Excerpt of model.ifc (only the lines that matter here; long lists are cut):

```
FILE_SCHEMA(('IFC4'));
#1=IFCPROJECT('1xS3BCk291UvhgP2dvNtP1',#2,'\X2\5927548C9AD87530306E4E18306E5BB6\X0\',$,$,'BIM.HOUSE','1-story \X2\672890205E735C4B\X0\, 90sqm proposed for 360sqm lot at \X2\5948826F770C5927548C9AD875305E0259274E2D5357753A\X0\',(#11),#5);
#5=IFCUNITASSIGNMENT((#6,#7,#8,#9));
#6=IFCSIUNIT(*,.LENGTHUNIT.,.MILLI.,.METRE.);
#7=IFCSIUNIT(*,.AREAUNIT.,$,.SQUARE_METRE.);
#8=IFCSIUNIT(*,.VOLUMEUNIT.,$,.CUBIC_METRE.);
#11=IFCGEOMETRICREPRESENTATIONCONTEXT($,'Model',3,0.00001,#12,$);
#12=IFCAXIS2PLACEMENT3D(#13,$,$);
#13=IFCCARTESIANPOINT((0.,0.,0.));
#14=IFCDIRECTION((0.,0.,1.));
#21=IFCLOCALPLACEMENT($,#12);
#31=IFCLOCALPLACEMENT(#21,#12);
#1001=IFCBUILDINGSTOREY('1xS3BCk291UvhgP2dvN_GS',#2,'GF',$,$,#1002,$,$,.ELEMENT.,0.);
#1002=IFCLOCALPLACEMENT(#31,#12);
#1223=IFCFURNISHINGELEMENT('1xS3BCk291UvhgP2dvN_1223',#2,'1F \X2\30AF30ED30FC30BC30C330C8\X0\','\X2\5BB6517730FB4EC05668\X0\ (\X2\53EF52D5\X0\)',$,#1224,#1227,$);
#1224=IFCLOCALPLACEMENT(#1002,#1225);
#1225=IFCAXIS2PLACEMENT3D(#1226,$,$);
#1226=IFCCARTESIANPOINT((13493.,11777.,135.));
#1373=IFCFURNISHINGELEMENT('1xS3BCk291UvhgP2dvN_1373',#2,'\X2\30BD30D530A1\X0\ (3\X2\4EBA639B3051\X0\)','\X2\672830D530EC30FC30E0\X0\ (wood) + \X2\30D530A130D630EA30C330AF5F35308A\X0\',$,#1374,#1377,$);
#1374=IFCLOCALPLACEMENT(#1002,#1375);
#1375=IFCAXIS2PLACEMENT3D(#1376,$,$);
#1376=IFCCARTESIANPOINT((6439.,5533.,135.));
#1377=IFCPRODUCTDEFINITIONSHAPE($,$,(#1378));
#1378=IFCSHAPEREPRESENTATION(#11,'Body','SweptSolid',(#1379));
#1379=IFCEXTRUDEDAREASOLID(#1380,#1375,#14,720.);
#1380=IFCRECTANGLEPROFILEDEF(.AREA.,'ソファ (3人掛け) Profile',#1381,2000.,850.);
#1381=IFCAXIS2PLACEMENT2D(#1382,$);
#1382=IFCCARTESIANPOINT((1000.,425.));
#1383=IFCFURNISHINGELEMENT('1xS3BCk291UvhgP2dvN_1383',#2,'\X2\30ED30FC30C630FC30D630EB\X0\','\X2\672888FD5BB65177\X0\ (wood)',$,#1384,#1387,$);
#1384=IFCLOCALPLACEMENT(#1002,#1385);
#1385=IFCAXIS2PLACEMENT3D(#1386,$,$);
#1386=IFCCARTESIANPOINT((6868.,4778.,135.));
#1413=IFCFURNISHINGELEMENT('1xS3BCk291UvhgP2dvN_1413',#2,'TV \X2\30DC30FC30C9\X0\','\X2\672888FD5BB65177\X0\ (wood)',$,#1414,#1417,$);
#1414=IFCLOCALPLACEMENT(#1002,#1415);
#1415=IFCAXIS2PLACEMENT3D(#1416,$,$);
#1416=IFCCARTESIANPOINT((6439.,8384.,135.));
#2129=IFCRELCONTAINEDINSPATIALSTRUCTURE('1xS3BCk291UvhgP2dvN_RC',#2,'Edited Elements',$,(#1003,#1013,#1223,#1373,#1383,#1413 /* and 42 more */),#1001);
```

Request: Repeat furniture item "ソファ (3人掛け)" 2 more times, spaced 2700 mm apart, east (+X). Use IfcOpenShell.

```python
import numpy as np
import ifcopenshell
import ifcopenshell.api.geometry
import ifcopenshell.api.root
import ifcopenshell.util.element
import ifcopenshell.util.placement
import ifcopenshell.util.unit

model = ifcopenshell.open("model.ifc")
unit_scale = ifcopenshell.util.unit.calculate_unit_scale(model)


def reuse_history(source, copy):
    """copy_class also copies each property set's owner history, people and application; keep the originals."""
    for rel in copy.IsDefinedBy:
        if rel.is_a("IfcRelDefinesByProperties") and (history := rel.RelatingPropertyDefinition.OwnerHistory):
            rel.RelatingPropertyDefinition.OwnerHistory = source.OwnerHistory
            ifcopenshell.util.element.remove_deep2(model, history)


source = model.by_id(1373)
base = ifcopenshell.util.placement.get_local_placement(source.ObjectPlacement)
step = np.array([1.0, 0.0, 0.0]) * 2.7 / unit_scale

for i in range(1, 3):
    copy = ifcopenshell.api.root.copy_class(model, product=source)
    copy.Representation = ifcopenshell.util.element.copy_deep(
        model, source.Representation, exclude=["IfcGeometricRepresentationContext", "IfcRepresentationMap"]
    )
    reuse_history(source, copy)
    matrix = base.copy()
    matrix[:3, 3] += i * step
    print("added at", matrix[:3, 3].round(3) + 0.0)
    ifcopenshell.api.geometry.edit_object_placement(model, product=copy, matrix=matrix, is_si=False)

model.write("model_v2.ifc")
```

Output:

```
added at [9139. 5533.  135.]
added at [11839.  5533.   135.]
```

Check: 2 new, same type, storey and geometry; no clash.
